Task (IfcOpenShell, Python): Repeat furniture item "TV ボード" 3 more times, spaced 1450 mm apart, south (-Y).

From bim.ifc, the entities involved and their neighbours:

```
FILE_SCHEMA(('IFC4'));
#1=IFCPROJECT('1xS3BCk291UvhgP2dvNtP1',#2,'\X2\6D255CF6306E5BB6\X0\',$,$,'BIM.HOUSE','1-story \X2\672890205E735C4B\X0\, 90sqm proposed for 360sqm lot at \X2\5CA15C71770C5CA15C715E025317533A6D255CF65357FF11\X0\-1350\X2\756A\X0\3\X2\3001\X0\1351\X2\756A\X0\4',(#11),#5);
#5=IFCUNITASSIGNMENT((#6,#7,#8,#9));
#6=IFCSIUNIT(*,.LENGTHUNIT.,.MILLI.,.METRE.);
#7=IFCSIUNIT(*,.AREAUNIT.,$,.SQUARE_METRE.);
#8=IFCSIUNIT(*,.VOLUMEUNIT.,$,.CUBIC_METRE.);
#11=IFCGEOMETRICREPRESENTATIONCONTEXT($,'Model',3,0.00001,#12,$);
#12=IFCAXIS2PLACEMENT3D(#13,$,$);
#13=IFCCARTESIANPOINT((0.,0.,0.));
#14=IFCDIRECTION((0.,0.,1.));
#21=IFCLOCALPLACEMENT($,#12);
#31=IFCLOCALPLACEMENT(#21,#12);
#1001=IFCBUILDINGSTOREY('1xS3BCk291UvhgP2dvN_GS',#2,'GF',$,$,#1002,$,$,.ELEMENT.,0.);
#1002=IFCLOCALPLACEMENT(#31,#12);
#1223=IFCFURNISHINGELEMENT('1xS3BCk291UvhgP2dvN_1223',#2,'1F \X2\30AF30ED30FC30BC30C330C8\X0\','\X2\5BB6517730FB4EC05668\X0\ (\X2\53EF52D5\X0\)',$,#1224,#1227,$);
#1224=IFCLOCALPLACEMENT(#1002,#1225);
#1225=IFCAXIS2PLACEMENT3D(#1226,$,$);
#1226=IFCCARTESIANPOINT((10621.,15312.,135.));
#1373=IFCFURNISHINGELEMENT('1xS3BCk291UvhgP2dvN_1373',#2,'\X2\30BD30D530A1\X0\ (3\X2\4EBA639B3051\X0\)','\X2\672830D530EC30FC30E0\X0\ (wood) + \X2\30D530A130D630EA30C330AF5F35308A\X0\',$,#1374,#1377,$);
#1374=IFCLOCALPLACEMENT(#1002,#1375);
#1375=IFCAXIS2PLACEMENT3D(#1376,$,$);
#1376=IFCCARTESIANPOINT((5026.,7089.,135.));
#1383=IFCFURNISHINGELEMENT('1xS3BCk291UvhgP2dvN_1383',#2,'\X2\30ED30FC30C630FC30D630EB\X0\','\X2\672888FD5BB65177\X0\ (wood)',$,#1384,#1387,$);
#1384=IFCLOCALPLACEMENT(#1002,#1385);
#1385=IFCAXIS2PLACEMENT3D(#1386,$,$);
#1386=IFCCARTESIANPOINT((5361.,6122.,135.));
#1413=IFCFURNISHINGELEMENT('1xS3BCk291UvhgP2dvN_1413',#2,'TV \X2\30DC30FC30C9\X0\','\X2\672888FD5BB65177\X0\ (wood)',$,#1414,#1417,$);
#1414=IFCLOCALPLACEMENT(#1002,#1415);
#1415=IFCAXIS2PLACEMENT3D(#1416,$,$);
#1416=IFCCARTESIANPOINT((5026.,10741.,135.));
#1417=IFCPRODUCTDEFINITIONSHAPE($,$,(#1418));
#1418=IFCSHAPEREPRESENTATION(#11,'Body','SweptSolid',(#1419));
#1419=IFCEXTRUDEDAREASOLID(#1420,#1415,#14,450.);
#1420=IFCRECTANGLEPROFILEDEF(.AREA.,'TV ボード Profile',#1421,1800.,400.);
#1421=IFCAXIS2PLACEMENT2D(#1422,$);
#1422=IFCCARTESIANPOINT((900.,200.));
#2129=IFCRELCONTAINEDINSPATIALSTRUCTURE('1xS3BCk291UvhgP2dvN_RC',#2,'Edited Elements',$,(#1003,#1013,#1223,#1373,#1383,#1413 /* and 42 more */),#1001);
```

```python
import numpy as np
import ifcopenshell
import ifcopenshell.api.geometry
import ifcopenshell.api.root
import ifcopenshell.util.element
import ifcopenshell.util.placement

model = ifcopenshell.open("bim.ifc")


def reuse_history(source, copy):
    """copy_class also copies each property set's owner history, people and application; keep the originals."""
    for rel in copy.IsDefinedBy:
        if rel.is_a("IfcRelDefinesByProperties") and (history := rel.RelatingPropertyDefinition.OwnerHistory):
            rel.RelatingPropertyDefinition.OwnerHistory = source.OwnerHistory
            ifcopenshell.util.element.remove_deep2(model, history)


source = model.by_guid("1xS3BCk291UvhgP2dvN_1413")
base = ifcopenshell.util.placement.get_local_placement(source.ObjectPlacement)
step = np.array([0.0, -1.0, 0.0]) * 1450.0

for i in range(1, 4):
    copy = ifcopenshell.api.root.copy_class(model, product=source)
    copy.Representation = ifcopenshell.util.element.copy_deep(
        model, source.Representation, exclude=["IfcGeometricRepresentationContext", "IfcRepresentationMap"]
    )
    reuse_history(source, copy)
    matrix = base.copy()
    matrix[:3, 3] += i * step
    print("added at", matrix[:3, 3].round(3) + 0.0)
    ifcopenshell.api.geometry.edit_object_placement(model, product=copy, matrix=matrix, is_si=False)

model.write("bim-out.ifc")
```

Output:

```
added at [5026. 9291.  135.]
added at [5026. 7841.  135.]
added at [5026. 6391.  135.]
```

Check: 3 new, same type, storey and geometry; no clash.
